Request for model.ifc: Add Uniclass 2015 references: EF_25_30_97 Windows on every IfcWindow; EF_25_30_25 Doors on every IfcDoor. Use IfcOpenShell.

First a look at what the model holds.

```python
import ifcopenshell

model = ifcopenshell.open("model.ifc")
print(model.schema)
print("classifications:", [c.Name for c in model.by_type("IfcClassification")])
for ifc_class in ("IfcDoor", "IfcRoof", "IfcStair", "IfcWall", "IfcWindow"):
    print(ifc_class, len(model.by_type(ifc_class)))
```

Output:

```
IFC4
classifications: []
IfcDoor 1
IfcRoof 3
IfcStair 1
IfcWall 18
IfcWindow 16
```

```python
import ifcopenshell
import ifcopenshell.api.classification

model = ifcopenshell.open("model.ifc")

system = ifcopenshell.api.classification.add_classification(model, classification="Uniclass 2015")

codes = {
    "IfcWindow": ("EF_25_30_97", "Windows"),
    "IfcDoor": ("EF_25_30_25", "Doors"),
}
for ifc_class, (code, name) in codes.items():
    products = model.by_type(ifc_class)
    ifcopenshell.api.classification.add_reference(
        model, products=products, classification=system, identification=code, name=name
    )
    print(code, len(products))

model.write("model_updated.ifc")
```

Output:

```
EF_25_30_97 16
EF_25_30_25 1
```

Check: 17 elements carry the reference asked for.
